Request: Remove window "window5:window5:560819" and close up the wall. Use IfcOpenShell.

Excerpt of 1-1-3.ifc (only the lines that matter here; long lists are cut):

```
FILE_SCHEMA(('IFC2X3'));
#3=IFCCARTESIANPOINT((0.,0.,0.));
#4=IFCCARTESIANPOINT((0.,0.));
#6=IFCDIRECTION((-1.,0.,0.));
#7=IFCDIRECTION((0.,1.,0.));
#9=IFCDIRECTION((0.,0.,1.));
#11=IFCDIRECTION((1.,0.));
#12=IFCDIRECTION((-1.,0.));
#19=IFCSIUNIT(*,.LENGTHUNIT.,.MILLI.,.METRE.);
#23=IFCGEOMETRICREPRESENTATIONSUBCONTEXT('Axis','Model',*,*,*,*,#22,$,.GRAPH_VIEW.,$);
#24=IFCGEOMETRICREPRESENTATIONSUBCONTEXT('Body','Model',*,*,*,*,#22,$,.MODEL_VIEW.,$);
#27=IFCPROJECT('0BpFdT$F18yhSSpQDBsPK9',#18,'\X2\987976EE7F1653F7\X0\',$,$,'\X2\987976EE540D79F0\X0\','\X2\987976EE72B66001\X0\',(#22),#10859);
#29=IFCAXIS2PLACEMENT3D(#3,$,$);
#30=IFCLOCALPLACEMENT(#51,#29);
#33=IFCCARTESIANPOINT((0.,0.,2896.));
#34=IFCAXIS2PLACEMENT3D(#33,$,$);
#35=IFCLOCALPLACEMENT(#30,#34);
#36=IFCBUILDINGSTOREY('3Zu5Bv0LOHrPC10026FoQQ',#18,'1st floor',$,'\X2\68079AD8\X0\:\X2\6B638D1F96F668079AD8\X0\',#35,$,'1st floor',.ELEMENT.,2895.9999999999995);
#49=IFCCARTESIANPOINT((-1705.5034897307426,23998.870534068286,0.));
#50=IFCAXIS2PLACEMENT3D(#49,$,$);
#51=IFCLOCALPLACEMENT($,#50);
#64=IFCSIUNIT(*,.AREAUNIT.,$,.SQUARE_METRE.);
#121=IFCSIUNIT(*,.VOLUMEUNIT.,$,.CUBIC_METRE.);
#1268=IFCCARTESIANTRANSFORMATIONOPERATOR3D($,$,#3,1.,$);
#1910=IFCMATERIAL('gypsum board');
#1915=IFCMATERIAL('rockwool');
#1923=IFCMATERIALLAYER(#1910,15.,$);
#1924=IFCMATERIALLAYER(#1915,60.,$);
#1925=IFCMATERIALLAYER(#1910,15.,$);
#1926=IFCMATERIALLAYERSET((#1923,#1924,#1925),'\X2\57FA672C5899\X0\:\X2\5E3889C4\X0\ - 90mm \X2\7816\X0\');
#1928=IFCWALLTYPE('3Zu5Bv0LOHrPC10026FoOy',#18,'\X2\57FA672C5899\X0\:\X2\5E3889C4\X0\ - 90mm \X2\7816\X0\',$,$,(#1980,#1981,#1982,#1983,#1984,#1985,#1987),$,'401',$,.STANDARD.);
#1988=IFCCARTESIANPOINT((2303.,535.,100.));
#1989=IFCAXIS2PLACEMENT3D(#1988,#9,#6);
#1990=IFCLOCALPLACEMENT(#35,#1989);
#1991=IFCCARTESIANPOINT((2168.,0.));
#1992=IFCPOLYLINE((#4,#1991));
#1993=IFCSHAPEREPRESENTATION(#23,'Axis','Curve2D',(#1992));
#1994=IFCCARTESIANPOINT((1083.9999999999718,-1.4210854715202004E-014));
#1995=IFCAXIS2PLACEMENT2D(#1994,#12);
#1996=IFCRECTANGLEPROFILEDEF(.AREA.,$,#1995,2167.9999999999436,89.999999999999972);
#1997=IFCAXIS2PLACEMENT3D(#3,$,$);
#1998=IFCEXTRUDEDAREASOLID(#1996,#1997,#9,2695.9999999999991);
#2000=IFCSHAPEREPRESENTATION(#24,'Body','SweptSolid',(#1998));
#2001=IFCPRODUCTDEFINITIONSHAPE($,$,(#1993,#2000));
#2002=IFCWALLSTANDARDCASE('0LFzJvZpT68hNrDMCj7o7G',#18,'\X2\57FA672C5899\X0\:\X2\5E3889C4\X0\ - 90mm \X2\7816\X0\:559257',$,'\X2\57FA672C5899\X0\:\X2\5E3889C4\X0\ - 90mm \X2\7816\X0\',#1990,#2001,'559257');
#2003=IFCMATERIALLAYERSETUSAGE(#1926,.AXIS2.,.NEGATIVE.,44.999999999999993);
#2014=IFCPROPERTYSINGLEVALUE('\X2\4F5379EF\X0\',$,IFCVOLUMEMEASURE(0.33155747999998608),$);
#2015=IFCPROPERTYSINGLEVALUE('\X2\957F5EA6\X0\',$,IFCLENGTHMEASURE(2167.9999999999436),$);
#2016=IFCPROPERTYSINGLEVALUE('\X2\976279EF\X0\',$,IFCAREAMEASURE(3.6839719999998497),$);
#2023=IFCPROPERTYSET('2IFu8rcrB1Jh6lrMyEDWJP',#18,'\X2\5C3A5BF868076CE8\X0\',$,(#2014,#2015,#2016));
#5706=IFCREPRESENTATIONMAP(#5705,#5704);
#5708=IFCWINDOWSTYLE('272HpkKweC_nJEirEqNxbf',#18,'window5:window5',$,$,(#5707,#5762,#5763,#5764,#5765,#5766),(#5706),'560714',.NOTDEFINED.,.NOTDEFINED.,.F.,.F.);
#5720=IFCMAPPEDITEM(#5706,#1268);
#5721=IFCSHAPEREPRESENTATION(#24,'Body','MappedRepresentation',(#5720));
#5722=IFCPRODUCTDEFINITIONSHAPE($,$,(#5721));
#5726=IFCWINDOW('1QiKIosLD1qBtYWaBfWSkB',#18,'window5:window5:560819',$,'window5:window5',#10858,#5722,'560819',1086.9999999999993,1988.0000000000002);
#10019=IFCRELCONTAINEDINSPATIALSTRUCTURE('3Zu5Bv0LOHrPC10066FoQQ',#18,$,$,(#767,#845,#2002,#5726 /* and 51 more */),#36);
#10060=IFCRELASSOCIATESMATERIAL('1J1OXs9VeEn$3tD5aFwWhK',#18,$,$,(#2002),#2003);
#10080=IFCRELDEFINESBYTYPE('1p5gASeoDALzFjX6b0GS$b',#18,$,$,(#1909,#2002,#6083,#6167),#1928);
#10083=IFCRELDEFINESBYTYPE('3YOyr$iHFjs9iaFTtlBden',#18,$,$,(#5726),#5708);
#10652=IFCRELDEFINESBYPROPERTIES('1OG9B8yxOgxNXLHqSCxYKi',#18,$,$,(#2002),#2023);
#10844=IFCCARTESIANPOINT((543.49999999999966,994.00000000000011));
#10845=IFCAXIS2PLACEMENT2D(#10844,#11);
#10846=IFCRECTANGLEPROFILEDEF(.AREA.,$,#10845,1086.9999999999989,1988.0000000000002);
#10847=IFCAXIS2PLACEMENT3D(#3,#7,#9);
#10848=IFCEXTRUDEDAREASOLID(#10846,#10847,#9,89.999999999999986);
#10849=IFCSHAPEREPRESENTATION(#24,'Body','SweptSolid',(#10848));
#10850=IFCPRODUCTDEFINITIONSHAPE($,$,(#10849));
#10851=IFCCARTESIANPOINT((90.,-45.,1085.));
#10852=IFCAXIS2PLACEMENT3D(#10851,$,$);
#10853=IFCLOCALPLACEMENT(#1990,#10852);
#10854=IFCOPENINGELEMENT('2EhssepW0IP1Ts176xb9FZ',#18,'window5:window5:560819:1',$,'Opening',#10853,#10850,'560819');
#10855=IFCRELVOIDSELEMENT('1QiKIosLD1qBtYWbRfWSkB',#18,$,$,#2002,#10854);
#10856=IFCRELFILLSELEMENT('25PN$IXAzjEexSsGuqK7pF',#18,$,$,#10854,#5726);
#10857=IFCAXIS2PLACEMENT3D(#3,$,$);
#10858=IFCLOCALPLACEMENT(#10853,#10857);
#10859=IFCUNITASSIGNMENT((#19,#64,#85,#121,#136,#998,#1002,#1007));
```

```python
import ifcopenshell
import ifcopenshell.api.feature
import ifcopenshell.api.pset
import ifcopenshell.api.root
import ifcopenshell.geom
import ifcopenshell.util.element
import ifcopenshell.util.shape
import ifcopenshell.util.unit

model = ifcopenshell.open("1-1-3.ifc")
area_scale = ifcopenshell.util.unit.calculate_unit_scale(model, "AREAUNIT")
volume_scale = ifcopenshell.util.unit.calculate_unit_scale(model, "VOLUMEUNIT")
settings = ifcopenshell.geom.settings()


def volume(element):
    """Net volume in cubic metres, openings subtracted."""
    shape = ifcopenshell.geom.create_shape(settings, element)
    return ifcopenshell.util.shape.get_volume(shape.geometry)


window = model.by_guid("1QiKIosLD1qBtYWaBfWSkB")
opening = window.FillsVoids[0].RelatingOpeningElement
wall = opening.VoidsElements[0].RelatingBuildingElement
before = volume(wall)

ifcopenshell.api.root.remove_product(model, product=window)
ifcopenshell.api.feature.remove_feature(model, feature=opening)

after = volume(wall)
thickness = 0.09  # wall thickness in metres

# Update the wall's stored quantities.
pset = model.by_id(ifcopenshell.util.element.get_pset(wall, "尺寸标注", should_inherit=False)["id"])
ifcopenshell.api.pset.edit_pset(model, pset=pset, properties={
    "体积": model.create_entity("IfcVolumeMeasure", after / volume_scale),
    "面积": model.create_entity("IfcAreaMeasure", after / thickness / area_scale),
})

print(f"wall volume {before:.3f} -> {after:.3f} m3")

model.write("1-1-3-out.ifc")
```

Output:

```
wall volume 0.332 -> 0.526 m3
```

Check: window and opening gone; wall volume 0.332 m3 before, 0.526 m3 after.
